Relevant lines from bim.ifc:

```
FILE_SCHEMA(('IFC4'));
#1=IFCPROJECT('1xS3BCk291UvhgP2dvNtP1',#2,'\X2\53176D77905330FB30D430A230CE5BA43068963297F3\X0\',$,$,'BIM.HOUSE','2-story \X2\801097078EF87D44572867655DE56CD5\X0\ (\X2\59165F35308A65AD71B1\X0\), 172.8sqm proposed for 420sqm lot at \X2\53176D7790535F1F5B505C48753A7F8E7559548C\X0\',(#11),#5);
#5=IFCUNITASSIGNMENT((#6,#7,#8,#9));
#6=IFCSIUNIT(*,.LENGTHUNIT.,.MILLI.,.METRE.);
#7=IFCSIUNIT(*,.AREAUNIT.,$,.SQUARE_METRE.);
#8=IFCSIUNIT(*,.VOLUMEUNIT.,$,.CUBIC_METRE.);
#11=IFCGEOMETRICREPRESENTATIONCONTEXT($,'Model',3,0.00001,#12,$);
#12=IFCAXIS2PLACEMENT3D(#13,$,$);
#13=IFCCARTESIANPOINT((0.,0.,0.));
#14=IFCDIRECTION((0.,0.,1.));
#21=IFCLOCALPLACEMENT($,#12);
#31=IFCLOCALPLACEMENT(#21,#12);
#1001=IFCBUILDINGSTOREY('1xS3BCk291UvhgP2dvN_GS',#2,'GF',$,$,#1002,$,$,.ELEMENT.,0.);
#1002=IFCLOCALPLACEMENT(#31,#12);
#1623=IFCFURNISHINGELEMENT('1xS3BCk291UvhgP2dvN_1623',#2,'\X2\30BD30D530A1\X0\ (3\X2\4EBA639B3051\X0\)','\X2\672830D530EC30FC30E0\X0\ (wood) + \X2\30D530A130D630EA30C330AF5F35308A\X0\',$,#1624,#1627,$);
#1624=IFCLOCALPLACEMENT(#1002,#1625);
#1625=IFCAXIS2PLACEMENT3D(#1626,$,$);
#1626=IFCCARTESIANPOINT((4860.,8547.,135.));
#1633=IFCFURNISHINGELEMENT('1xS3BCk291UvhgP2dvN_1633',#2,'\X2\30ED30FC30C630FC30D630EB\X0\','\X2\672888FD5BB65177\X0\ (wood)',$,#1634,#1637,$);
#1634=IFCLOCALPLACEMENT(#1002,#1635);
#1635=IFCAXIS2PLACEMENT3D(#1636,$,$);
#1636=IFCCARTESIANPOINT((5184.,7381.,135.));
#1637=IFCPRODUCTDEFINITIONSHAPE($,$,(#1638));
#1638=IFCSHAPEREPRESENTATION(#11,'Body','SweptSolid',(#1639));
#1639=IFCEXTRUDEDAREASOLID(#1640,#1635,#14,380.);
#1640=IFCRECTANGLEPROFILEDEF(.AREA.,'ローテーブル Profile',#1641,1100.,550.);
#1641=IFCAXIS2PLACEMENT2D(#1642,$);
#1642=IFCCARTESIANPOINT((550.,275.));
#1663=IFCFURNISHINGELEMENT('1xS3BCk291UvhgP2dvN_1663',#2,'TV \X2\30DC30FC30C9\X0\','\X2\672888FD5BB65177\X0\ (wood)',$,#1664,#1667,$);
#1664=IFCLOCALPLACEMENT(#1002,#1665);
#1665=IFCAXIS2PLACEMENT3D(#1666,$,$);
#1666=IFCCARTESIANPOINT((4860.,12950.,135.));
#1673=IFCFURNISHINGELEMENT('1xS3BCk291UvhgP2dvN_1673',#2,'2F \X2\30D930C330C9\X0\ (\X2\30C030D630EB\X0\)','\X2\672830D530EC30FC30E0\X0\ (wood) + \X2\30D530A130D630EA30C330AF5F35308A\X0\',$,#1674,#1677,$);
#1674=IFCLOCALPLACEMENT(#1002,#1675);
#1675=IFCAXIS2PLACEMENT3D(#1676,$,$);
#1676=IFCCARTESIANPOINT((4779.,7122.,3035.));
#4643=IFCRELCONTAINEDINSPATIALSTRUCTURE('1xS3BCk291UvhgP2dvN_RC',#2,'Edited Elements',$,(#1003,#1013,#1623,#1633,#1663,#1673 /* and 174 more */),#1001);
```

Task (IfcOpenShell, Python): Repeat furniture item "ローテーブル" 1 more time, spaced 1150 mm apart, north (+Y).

```python
import numpy as np
import ifcopenshell
import ifcopenshell.api.geometry
import ifcopenshell.api.root
import ifcopenshell.util.element
import ifcopenshell.util.placement

model = ifcopenshell.open("bim.ifc")


def reuse_history(source, copy):
    """copy_class also copies each property set's owner history, people and application; keep the originals."""
    for rel in copy.IsDefinedBy:
        if rel.is_a("IfcRelDefinesByProperties") and (history := rel.RelatingPropertyDefinition.OwnerHistory):
            rel.RelatingPropertyDefinition.OwnerHistory = source.OwnerHistory
            ifcopenshell.util.element.remove_deep2(model, history)


source = model.by_id(1633)
base = ifcopenshell.util.placement.get_local_placement(source.ObjectPlacement)
step = np.array([0.0, 1.0, 0.0]) * 1150.0

for i in range(1, 2):
    copy = ifcopenshell.api.root.copy_class(model, product=source)
    copy.Representation = ifcopenshell.util.element.copy_deep(
        model, source.Representation, exclude=["IfcGeometricRepresentationContext", "IfcRepresentationMap"]
    )
    reuse_history(source, copy)
    matrix = base.copy()
    matrix[:3, 3] += i * step
    print("added at", matrix[:3, 3].round(3) + 0.0)
    ifcopenshell.api.geometry.edit_object_placement(model, product=copy, matrix=matrix, is_si=False)

model.write("bim_v2.ifc")
```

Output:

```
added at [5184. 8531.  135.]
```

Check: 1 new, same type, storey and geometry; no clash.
